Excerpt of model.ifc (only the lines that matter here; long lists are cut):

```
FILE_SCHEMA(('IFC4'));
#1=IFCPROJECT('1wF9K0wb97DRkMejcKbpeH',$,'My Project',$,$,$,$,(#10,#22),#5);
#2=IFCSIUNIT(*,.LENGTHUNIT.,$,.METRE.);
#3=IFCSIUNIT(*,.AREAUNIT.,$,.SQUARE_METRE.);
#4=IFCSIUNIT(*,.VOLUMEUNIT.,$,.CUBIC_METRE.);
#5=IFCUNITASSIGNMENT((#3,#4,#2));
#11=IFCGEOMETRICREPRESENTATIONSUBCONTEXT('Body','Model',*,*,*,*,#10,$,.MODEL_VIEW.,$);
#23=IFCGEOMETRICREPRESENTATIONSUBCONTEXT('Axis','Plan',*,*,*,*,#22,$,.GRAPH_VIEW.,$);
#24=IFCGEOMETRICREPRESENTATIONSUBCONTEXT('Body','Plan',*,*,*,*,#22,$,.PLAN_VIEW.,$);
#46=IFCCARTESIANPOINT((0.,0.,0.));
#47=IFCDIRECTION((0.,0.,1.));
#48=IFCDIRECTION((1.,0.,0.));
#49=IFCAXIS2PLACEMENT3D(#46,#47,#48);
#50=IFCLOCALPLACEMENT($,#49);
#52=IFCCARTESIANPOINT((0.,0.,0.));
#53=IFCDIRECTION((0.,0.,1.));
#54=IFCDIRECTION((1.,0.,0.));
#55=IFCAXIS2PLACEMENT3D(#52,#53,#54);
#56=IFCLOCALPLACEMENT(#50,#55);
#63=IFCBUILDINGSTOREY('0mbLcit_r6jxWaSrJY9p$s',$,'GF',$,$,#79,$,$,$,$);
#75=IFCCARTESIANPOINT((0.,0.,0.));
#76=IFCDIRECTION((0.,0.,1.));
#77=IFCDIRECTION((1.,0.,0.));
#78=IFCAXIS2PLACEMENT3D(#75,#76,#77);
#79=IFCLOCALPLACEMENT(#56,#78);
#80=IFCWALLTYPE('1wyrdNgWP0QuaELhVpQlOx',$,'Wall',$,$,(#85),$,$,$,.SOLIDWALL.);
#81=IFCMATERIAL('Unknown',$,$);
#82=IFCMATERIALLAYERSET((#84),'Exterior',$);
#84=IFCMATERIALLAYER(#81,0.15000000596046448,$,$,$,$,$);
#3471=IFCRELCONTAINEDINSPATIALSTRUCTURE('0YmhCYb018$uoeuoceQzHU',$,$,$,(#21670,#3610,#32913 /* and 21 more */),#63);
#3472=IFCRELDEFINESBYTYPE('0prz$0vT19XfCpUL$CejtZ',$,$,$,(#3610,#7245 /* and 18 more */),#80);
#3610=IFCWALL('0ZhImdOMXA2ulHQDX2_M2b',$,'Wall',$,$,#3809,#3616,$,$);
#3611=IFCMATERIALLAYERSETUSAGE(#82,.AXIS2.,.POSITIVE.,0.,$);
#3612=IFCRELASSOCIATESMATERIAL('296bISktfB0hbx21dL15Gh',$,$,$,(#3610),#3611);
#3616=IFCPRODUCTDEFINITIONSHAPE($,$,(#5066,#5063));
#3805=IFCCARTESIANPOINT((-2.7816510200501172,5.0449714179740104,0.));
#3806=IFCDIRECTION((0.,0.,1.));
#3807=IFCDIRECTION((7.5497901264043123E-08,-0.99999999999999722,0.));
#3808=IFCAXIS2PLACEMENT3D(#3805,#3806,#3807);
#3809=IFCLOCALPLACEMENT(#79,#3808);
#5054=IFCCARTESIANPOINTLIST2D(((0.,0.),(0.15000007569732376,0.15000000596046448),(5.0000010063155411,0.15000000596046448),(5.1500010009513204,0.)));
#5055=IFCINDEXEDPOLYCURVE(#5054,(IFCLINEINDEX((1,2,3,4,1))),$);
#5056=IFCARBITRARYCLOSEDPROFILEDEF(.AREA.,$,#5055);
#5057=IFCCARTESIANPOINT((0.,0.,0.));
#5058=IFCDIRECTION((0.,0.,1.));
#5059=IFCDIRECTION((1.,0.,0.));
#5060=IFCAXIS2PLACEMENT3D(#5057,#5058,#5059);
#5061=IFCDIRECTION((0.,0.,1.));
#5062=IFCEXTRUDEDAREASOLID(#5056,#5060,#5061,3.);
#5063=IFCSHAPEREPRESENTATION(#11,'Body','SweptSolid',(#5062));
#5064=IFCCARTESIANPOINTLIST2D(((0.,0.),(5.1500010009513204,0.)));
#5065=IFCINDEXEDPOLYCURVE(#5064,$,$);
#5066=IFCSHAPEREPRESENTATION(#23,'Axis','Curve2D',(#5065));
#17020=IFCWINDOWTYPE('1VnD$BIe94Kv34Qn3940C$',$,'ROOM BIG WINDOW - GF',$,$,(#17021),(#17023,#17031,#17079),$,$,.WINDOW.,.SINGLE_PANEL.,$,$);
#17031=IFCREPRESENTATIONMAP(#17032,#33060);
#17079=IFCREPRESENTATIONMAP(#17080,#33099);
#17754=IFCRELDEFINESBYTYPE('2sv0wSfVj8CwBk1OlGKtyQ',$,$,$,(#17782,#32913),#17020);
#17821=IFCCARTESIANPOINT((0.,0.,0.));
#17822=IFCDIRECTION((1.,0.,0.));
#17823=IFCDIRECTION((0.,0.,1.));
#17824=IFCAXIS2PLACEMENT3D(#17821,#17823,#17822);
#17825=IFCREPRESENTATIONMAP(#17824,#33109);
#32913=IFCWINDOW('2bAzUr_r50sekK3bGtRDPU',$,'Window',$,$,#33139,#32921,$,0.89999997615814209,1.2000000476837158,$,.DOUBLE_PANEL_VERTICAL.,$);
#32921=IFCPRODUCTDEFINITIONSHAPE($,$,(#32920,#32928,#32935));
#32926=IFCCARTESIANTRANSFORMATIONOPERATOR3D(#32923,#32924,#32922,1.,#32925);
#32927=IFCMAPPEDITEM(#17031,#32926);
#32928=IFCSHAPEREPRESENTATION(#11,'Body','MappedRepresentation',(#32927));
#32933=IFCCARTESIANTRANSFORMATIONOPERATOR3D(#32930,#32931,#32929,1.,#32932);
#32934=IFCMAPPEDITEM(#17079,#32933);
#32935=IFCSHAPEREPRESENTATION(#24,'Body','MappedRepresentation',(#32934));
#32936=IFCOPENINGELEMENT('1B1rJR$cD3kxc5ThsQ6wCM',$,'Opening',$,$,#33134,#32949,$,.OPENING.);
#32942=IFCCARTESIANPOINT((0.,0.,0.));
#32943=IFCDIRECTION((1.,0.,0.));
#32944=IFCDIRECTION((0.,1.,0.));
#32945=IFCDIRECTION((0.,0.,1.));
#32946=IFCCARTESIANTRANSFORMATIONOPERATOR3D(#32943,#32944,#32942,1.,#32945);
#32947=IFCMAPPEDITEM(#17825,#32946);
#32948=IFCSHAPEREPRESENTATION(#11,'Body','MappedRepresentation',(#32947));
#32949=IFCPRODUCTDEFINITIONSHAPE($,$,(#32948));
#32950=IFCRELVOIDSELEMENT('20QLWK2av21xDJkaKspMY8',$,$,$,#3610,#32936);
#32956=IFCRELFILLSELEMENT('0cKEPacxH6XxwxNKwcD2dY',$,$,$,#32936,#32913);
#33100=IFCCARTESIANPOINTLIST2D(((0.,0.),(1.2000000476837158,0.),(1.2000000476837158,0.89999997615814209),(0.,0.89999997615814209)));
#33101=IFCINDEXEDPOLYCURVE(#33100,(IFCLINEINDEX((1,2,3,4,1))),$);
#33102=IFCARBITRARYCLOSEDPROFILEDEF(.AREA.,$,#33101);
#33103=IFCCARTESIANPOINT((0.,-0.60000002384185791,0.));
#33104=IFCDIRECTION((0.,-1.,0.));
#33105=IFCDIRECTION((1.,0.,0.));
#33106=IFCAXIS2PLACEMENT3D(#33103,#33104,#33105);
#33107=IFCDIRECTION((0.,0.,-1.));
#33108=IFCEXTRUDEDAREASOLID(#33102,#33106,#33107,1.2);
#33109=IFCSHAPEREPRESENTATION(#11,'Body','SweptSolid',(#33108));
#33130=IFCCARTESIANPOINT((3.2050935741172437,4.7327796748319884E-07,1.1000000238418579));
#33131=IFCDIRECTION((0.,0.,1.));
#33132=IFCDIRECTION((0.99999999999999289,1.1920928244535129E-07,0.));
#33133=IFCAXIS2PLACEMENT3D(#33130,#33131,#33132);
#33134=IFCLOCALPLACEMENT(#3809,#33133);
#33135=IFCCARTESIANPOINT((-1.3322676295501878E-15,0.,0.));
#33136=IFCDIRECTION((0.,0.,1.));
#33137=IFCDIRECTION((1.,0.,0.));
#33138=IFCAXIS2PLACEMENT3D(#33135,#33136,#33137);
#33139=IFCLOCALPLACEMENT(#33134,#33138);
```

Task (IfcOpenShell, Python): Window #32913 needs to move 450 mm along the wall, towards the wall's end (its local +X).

```python
import ifcopenshell
import ifcopenshell.api.geometry
import ifcopenshell.util.placement
import ifcopenshell.util.unit

model = ifcopenshell.open("model.ifc")
unit_scale = ifcopenshell.util.unit.calculate_unit_scale(model)

window = model.by_id(32913)
opening = window.FillsVoids[0].RelatingOpeningElement
wall = opening.VoidsElements[0].RelatingBuildingElement

wall_matrix = ifcopenshell.util.placement.get_local_placement(wall.ObjectPlacement)
shift = wall_matrix[:3, 0] * 0.45 / unit_scale
before = ifcopenshell.util.placement.get_local_placement(window.ObjectPlacement)[:3, 3].copy()

# The window is placed relative to its opening, so it follows when the opening moves.
matrix = ifcopenshell.util.placement.get_local_placement(opening.ObjectPlacement)
matrix[:3, 3] += shift
ifcopenshell.api.geometry.edit_object_placement(
    model, product=opening, matrix=matrix, is_si=False, should_transform_children=True
)

after = ifcopenshell.util.placement.get_local_placement(window.ObjectPlacement)[:3, 3]
print("window moved by", (after - before).round(3) + 0.0)

model.write("model_updated.ifc")
```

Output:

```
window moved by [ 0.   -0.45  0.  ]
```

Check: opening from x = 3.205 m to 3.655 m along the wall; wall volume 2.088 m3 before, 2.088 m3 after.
